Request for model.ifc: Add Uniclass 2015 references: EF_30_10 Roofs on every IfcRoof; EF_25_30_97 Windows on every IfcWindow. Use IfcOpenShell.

First a look at what the model holds.

```python
import ifcopenshell

model = ifcopenshell.open("model.ifc")
print(model.schema)
print("classifications:", [c.Name for c in model.by_type("IfcClassification")])
for ifc_class in ("IfcDoor", "IfcRoof", "IfcStair", "IfcWall", "IfcWindow"):
    print(ifc_class, len(model.by_type(ifc_class)))
```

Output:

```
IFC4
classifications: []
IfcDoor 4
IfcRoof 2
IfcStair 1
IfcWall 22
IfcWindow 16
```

```python
import ifcopenshell
import ifcopenshell.api.classification

model = ifcopenshell.open("model.ifc")

system = ifcopenshell.api.classification.add_classification(model, classification="Uniclass 2015")

codes = {
    "IfcRoof": ("EF_30_10", "Roofs"),
    "IfcWindow": ("EF_25_30_97", "Windows"),
}
for ifc_class, (code, name) in codes.items():
    products = model.by_type(ifc_class)
    ifcopenshell.api.classification.add_reference(
        model, products=products, classification=system, identification=code, name=name
    )
    print(code, len(products))

model.write("model_edited.ifc")
```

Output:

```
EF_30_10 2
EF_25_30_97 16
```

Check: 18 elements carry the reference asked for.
